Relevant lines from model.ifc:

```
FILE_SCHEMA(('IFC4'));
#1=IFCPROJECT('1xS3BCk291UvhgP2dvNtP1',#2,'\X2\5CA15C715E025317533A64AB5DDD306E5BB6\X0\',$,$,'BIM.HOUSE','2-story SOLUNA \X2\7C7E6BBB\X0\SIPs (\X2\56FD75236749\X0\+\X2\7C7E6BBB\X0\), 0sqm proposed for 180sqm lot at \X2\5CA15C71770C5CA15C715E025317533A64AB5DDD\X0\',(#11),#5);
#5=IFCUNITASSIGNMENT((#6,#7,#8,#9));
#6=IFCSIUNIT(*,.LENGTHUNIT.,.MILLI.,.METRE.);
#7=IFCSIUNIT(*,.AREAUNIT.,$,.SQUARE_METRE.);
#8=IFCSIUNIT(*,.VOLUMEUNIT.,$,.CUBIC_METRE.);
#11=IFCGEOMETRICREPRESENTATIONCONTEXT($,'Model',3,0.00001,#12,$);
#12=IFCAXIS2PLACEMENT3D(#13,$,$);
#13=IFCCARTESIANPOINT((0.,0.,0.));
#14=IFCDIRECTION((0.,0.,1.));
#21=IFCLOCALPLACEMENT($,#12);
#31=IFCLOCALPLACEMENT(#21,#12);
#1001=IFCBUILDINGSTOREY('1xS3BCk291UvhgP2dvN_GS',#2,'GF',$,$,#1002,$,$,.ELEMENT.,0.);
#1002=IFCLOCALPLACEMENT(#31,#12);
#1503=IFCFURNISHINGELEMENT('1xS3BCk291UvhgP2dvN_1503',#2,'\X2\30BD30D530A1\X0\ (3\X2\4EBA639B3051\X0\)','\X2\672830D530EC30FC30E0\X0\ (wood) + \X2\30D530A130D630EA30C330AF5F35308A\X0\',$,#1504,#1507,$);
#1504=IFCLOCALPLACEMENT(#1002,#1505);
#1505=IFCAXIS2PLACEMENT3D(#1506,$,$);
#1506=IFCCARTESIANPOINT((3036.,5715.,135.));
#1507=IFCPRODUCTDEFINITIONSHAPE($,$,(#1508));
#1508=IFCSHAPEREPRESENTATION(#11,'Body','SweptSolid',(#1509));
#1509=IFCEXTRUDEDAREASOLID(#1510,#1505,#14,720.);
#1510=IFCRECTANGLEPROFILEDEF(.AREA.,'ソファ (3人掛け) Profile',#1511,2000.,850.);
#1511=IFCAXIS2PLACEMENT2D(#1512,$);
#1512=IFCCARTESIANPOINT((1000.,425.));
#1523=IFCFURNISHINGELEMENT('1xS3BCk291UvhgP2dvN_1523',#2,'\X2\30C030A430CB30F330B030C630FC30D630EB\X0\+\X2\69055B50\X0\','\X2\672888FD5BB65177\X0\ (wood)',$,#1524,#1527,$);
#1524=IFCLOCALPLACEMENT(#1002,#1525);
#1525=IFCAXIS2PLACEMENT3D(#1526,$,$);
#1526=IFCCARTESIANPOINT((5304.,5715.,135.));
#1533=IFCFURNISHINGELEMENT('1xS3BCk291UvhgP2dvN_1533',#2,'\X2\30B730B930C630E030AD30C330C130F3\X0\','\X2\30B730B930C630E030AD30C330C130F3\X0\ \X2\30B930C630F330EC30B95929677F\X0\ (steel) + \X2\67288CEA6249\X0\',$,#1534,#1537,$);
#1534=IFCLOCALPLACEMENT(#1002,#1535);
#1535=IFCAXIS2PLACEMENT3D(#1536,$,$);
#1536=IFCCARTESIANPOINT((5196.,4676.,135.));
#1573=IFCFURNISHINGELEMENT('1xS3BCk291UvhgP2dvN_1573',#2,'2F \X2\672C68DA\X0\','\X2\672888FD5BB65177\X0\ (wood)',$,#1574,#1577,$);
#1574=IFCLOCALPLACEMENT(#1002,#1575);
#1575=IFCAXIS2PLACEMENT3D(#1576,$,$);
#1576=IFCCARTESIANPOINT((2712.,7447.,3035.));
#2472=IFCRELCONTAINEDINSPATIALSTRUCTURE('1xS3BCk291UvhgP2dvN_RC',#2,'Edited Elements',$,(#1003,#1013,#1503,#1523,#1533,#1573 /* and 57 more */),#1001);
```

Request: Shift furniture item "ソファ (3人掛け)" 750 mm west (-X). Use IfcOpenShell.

```python
import ifcopenshell
import ifcopenshell.api.geometry
import ifcopenshell.util.placement
import ifcopenshell.util.unit

model = ifcopenshell.open("model.ifc")
unit_scale = ifcopenshell.util.unit.calculate_unit_scale(model)

item = model.by_guid("1xS3BCk291UvhgP2dvN_1503")
matrix = ifcopenshell.util.placement.get_local_placement(item.ObjectPlacement)
matrix[0, 3] -= 0.75 / unit_scale
ifcopenshell.api.geometry.edit_object_placement(model, product=item, matrix=matrix, is_si=False)

print(ifcopenshell.util.placement.get_local_placement(item.ObjectPlacement).round(3) + 0.0)

model.write("model_rev.ifc")
```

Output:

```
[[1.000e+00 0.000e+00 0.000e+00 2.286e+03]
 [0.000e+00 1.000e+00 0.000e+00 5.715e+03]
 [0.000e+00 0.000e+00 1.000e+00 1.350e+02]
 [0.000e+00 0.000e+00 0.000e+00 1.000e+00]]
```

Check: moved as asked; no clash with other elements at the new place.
